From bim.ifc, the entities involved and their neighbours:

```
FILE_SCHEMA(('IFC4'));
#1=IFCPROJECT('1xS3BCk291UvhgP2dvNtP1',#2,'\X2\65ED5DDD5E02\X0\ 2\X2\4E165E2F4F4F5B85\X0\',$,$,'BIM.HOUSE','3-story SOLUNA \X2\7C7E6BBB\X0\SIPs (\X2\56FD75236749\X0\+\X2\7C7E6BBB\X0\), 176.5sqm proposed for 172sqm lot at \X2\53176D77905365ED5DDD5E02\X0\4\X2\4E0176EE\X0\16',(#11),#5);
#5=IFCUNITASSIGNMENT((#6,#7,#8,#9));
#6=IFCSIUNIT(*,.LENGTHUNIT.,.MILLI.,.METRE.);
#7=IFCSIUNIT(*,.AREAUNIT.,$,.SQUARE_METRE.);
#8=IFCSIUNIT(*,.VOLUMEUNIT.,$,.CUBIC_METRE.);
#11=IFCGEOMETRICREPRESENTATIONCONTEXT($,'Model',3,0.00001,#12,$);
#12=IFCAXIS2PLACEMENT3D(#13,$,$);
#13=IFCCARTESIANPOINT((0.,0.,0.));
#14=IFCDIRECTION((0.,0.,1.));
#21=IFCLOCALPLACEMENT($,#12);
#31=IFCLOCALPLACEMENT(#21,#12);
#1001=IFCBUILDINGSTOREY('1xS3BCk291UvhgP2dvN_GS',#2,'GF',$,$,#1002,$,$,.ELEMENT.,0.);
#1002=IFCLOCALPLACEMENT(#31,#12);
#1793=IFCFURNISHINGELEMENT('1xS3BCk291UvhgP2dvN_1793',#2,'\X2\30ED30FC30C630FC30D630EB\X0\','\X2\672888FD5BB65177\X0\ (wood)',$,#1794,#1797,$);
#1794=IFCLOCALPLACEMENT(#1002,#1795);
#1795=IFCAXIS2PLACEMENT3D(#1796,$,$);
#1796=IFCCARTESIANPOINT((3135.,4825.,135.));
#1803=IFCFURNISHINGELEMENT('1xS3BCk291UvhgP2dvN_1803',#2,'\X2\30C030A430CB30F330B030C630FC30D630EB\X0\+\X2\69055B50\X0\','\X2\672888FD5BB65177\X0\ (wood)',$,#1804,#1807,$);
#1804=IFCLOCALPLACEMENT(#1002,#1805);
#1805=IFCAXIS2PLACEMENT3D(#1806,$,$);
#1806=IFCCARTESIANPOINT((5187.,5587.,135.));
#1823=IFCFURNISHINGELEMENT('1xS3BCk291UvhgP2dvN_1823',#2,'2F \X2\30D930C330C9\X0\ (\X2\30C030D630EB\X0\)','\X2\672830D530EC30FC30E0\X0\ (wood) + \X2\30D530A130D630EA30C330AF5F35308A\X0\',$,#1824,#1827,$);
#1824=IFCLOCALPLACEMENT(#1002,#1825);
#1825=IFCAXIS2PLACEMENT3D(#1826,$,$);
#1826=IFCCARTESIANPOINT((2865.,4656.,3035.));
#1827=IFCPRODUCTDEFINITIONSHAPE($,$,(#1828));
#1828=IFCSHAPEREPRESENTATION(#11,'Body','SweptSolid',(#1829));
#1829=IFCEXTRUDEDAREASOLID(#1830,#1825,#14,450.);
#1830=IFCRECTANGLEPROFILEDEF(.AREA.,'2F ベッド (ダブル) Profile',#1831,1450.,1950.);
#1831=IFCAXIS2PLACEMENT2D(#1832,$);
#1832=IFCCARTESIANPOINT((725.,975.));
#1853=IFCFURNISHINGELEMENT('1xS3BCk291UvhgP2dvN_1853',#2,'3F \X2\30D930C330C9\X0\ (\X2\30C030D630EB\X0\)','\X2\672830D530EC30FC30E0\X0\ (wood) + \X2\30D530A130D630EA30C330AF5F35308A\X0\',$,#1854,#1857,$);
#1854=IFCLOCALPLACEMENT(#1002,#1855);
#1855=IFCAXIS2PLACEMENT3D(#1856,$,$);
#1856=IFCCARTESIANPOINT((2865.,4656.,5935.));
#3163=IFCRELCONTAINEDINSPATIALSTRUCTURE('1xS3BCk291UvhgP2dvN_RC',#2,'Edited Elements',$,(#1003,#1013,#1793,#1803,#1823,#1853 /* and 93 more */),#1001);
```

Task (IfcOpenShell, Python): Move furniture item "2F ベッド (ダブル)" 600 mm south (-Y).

```python
import ifcopenshell
import ifcopenshell.api.geometry
import ifcopenshell.util.placement

model = ifcopenshell.open("bim.ifc")

item = model.by_guid("1xS3BCk291UvhgP2dvN_1823")
matrix = ifcopenshell.util.placement.get_local_placement(item.ObjectPlacement)
matrix[1, 3] -= 600.0
ifcopenshell.api.geometry.edit_object_placement(model, product=item, matrix=matrix, is_si=False)

print(ifcopenshell.util.placement.get_local_placement(item.ObjectPlacement).round(3) + 0.0)

model.write("bim_updated.ifc")
```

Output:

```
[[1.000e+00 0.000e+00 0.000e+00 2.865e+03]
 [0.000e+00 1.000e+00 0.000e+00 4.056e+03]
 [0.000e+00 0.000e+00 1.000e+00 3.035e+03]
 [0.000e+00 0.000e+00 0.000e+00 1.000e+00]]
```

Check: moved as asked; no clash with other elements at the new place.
